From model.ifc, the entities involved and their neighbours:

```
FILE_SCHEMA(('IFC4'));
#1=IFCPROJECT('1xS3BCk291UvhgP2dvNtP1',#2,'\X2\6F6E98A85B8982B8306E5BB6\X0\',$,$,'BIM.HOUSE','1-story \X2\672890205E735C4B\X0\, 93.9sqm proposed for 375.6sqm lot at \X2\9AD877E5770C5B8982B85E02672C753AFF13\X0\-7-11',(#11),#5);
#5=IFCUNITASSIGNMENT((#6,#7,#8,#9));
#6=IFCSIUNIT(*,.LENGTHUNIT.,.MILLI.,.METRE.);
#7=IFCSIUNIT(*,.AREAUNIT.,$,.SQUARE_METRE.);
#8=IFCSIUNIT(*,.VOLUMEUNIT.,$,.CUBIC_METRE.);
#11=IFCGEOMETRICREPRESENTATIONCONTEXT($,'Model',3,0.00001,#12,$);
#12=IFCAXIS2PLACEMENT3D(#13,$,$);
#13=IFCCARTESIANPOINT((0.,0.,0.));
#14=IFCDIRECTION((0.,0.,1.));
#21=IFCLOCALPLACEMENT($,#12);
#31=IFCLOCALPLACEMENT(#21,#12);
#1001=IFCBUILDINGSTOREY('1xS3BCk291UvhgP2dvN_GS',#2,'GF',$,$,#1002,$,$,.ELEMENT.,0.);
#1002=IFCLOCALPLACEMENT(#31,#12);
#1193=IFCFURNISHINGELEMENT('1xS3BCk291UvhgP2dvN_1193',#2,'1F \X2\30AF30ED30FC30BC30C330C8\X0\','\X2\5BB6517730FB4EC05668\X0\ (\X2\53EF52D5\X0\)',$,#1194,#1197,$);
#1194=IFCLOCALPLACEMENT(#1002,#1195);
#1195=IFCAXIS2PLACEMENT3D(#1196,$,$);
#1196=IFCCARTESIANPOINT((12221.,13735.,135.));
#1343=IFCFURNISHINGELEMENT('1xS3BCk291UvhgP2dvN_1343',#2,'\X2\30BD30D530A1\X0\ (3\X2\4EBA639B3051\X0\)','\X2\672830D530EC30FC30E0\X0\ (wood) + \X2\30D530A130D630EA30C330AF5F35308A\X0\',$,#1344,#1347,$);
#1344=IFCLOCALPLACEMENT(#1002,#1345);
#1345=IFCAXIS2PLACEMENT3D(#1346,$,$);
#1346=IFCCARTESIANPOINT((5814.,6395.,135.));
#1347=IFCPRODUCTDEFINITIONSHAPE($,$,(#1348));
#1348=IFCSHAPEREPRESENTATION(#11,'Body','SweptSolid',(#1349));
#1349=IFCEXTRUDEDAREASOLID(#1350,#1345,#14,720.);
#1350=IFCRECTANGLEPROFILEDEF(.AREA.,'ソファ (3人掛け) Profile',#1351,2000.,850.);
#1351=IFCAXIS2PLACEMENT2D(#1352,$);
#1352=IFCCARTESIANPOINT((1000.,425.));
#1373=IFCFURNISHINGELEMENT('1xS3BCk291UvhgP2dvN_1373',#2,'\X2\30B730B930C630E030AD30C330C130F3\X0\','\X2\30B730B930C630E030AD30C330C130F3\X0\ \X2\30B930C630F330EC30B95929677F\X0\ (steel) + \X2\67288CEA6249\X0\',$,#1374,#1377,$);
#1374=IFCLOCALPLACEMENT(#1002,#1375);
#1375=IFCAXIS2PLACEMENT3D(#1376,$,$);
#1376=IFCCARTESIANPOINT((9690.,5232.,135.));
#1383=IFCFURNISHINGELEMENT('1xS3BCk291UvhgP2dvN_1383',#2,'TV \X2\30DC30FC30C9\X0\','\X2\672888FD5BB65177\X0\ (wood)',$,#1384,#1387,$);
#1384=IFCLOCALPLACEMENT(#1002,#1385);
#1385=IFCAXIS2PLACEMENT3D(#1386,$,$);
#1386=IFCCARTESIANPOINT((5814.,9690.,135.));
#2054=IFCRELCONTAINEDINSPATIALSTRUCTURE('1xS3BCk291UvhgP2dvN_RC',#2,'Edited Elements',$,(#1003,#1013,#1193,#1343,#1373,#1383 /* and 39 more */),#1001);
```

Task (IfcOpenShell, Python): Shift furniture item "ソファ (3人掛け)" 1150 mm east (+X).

```python
import ifcopenshell
import ifcopenshell.api.geometry
import ifcopenshell.util.placement

model = ifcopenshell.open("model.ifc")

item = model.by_id(1343)
matrix = ifcopenshell.util.placement.get_local_placement(item.ObjectPlacement)
matrix[0, 3] += 1150.0
ifcopenshell.api.geometry.edit_object_placement(model, product=item, matrix=matrix, is_si=False)

print(ifcopenshell.util.placement.get_local_placement(item.ObjectPlacement).round(3) + 0.0)

model.write("model_v2.ifc")
```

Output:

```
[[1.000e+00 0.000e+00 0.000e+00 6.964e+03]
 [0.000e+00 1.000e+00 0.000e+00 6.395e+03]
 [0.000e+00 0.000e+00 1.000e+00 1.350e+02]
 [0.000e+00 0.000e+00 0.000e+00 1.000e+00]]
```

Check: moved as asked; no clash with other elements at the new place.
